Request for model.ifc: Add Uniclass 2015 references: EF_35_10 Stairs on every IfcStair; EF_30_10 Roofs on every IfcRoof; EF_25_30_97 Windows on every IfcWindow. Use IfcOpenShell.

First a look at what the model holds.

```python
import ifcopenshell

model = ifcopenshell.open("model.ifc")
print(model.schema)
print("classifications:", [c.Name for c in model.by_type("IfcClassification")])
for ifc_class in ("IfcDoor", "IfcRoof", "IfcStair", "IfcWall", "IfcWindow"):
    print(ifc_class, len(model.by_type(ifc_class)))
```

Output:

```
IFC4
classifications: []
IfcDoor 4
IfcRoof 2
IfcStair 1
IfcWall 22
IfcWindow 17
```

```python
import ifcopenshell
import ifcopenshell.api.classification

model = ifcopenshell.open("model.ifc")

system = ifcopenshell.api.classification.add_classification(model, classification="Uniclass 2015")

codes = {
    "IfcStair": ("EF_35_10", "Stairs"),
    "IfcRoof": ("EF_30_10", "Roofs"),
    "IfcWindow": ("EF_25_30_97", "Windows"),
}
for ifc_class, (code, name) in codes.items():
    products = model.by_type(ifc_class)
    ifcopenshell.api.classification.add_reference(
        model, products=products, classification=system, identification=code, name=name
    )
    print(code, len(products))

model.write("model_rev.ifc")
```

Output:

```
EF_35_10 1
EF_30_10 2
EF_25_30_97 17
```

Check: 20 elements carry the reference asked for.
